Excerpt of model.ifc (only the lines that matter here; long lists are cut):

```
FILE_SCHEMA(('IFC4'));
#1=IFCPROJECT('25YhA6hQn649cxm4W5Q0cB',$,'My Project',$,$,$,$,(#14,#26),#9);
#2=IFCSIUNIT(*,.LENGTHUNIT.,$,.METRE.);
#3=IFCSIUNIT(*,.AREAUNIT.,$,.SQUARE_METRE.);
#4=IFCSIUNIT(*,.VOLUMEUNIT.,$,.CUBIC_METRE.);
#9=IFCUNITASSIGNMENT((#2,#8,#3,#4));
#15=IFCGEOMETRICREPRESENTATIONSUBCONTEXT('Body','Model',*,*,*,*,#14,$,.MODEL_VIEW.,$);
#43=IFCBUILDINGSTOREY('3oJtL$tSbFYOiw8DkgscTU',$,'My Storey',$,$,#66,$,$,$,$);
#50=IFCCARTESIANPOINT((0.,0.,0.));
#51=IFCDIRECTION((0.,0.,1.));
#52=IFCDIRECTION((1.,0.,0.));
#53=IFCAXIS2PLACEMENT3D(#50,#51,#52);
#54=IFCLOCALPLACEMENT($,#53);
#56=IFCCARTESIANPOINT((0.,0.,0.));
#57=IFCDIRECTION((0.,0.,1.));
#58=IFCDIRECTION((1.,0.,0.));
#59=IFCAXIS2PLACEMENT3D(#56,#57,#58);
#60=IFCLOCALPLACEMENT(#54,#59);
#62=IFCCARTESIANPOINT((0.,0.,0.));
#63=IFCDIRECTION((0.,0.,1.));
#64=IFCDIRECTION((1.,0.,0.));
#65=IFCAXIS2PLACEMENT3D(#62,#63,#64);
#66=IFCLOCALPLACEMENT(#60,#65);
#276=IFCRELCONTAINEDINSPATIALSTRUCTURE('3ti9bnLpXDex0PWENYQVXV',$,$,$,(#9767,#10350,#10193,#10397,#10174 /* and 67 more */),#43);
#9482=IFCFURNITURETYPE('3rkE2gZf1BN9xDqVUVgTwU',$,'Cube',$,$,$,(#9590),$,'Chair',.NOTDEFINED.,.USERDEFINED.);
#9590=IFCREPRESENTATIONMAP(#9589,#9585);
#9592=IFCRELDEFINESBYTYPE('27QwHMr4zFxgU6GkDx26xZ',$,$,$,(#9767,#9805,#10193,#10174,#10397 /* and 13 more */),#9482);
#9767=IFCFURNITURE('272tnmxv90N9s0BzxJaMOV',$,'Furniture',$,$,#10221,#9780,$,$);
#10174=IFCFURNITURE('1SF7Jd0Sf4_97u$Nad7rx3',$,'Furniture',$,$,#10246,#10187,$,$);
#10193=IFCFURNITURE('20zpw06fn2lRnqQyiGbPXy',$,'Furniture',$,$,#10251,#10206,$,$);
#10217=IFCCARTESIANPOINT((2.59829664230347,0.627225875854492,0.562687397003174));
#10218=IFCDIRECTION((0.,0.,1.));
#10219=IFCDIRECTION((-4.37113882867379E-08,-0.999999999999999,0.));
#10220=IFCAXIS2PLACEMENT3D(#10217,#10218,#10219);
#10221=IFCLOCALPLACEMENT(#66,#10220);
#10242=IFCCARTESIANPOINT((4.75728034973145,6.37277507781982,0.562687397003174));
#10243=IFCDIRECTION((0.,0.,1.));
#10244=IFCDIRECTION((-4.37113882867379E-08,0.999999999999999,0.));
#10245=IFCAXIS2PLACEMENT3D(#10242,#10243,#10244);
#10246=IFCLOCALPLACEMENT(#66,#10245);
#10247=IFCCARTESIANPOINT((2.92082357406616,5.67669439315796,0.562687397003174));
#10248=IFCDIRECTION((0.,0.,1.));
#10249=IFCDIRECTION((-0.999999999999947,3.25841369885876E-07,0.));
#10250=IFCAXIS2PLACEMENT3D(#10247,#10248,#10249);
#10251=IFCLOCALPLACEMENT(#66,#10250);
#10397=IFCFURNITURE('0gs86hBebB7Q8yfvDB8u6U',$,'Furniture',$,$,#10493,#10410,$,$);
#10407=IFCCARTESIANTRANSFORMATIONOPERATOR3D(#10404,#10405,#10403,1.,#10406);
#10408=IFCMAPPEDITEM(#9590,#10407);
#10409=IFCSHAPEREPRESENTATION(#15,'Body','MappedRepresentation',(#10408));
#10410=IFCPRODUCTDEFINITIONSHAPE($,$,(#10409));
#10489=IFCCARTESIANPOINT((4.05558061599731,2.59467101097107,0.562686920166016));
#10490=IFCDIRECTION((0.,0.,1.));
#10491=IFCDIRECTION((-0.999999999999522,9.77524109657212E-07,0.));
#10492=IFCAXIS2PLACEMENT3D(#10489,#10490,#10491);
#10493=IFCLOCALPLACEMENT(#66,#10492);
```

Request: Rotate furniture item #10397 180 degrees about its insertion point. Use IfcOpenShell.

```python
import ifcopenshell
import ifcopenshell.api.geometry
import ifcopenshell.util.placement

model = ifcopenshell.open("model.ifc")

item = model.by_guid("0gs86hBebB7Q8yfvDB8u6U")
matrix = ifcopenshell.util.placement.get_local_placement(item.ObjectPlacement)
matrix = matrix @ ifcopenshell.util.placement.rotation(180, "Z")
ifcopenshell.api.geometry.edit_object_placement(model, product=item, matrix=matrix, is_si=False)

print(ifcopenshell.util.placement.get_local_placement(item.ObjectPlacement).round(3) + 0.0)

model.write("model-out.ifc")
```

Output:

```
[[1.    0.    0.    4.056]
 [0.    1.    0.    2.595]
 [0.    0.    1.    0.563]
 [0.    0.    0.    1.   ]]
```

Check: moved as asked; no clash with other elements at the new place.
